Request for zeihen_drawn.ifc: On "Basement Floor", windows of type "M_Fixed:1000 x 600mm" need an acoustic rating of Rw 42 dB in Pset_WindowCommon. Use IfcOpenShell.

First a look at what the model holds.

```python
import ifcopenshell
import ifcopenshell.util.element

model = ifcopenshell.open("zeihen_drawn.ifc")
print(model.schema)
storey = next(s for s in model.by_type("IfcBuildingStorey") if s.Name == "Basement Floor")
windows = [e for e in ifcopenshell.util.element.get_decomposition(storey) if e.is_a("IfcWindow")]
seen = {}
for e in windows:
    element_type = ifcopenshell.util.element.get_type(e)
    key = (element_type.Name if element_type != e and element_type else None, ifcopenshell.util.element.get_pset(e, "Pset_WindowCommon", "AcousticRating"))
    seen[key] = seen.get(key, 0) + 1
for (name, value), count in sorted(seen.items(), key=str):
    print(count, "x", name, "|", value)
```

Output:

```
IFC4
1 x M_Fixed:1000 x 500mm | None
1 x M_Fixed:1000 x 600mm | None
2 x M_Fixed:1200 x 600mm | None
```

```python
import ifcopenshell
import ifcopenshell.api.pset
import ifcopenshell.util.element

model = ifcopenshell.open("zeihen_drawn.ifc")

storey = next(s for s in model.by_type("IfcBuildingStorey") if s.Name == "Basement Floor")
windows = [e for e in ifcopenshell.util.element.get_decomposition(storey) if e.is_a("IfcWindow")]

count = 0
for e in windows:
    element_type = ifcopenshell.util.element.get_type(e)
    if element_type in (None, e) or element_type.Name != "M_Fixed:1000 x 600mm":
        continue
    # add_pset returns the element's existing set when there is one.
    pset = ifcopenshell.api.pset.add_pset(model, product=e, name="Pset_WindowCommon")
    ifcopenshell.api.pset.edit_pset(model, pset=pset, properties={"AcousticRating": "Rw 42 dB"})
    count += 1

print(count, "windows updated")

model.write("zeihen_drawn_updated.ifc")
```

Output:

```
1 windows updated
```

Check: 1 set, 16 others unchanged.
